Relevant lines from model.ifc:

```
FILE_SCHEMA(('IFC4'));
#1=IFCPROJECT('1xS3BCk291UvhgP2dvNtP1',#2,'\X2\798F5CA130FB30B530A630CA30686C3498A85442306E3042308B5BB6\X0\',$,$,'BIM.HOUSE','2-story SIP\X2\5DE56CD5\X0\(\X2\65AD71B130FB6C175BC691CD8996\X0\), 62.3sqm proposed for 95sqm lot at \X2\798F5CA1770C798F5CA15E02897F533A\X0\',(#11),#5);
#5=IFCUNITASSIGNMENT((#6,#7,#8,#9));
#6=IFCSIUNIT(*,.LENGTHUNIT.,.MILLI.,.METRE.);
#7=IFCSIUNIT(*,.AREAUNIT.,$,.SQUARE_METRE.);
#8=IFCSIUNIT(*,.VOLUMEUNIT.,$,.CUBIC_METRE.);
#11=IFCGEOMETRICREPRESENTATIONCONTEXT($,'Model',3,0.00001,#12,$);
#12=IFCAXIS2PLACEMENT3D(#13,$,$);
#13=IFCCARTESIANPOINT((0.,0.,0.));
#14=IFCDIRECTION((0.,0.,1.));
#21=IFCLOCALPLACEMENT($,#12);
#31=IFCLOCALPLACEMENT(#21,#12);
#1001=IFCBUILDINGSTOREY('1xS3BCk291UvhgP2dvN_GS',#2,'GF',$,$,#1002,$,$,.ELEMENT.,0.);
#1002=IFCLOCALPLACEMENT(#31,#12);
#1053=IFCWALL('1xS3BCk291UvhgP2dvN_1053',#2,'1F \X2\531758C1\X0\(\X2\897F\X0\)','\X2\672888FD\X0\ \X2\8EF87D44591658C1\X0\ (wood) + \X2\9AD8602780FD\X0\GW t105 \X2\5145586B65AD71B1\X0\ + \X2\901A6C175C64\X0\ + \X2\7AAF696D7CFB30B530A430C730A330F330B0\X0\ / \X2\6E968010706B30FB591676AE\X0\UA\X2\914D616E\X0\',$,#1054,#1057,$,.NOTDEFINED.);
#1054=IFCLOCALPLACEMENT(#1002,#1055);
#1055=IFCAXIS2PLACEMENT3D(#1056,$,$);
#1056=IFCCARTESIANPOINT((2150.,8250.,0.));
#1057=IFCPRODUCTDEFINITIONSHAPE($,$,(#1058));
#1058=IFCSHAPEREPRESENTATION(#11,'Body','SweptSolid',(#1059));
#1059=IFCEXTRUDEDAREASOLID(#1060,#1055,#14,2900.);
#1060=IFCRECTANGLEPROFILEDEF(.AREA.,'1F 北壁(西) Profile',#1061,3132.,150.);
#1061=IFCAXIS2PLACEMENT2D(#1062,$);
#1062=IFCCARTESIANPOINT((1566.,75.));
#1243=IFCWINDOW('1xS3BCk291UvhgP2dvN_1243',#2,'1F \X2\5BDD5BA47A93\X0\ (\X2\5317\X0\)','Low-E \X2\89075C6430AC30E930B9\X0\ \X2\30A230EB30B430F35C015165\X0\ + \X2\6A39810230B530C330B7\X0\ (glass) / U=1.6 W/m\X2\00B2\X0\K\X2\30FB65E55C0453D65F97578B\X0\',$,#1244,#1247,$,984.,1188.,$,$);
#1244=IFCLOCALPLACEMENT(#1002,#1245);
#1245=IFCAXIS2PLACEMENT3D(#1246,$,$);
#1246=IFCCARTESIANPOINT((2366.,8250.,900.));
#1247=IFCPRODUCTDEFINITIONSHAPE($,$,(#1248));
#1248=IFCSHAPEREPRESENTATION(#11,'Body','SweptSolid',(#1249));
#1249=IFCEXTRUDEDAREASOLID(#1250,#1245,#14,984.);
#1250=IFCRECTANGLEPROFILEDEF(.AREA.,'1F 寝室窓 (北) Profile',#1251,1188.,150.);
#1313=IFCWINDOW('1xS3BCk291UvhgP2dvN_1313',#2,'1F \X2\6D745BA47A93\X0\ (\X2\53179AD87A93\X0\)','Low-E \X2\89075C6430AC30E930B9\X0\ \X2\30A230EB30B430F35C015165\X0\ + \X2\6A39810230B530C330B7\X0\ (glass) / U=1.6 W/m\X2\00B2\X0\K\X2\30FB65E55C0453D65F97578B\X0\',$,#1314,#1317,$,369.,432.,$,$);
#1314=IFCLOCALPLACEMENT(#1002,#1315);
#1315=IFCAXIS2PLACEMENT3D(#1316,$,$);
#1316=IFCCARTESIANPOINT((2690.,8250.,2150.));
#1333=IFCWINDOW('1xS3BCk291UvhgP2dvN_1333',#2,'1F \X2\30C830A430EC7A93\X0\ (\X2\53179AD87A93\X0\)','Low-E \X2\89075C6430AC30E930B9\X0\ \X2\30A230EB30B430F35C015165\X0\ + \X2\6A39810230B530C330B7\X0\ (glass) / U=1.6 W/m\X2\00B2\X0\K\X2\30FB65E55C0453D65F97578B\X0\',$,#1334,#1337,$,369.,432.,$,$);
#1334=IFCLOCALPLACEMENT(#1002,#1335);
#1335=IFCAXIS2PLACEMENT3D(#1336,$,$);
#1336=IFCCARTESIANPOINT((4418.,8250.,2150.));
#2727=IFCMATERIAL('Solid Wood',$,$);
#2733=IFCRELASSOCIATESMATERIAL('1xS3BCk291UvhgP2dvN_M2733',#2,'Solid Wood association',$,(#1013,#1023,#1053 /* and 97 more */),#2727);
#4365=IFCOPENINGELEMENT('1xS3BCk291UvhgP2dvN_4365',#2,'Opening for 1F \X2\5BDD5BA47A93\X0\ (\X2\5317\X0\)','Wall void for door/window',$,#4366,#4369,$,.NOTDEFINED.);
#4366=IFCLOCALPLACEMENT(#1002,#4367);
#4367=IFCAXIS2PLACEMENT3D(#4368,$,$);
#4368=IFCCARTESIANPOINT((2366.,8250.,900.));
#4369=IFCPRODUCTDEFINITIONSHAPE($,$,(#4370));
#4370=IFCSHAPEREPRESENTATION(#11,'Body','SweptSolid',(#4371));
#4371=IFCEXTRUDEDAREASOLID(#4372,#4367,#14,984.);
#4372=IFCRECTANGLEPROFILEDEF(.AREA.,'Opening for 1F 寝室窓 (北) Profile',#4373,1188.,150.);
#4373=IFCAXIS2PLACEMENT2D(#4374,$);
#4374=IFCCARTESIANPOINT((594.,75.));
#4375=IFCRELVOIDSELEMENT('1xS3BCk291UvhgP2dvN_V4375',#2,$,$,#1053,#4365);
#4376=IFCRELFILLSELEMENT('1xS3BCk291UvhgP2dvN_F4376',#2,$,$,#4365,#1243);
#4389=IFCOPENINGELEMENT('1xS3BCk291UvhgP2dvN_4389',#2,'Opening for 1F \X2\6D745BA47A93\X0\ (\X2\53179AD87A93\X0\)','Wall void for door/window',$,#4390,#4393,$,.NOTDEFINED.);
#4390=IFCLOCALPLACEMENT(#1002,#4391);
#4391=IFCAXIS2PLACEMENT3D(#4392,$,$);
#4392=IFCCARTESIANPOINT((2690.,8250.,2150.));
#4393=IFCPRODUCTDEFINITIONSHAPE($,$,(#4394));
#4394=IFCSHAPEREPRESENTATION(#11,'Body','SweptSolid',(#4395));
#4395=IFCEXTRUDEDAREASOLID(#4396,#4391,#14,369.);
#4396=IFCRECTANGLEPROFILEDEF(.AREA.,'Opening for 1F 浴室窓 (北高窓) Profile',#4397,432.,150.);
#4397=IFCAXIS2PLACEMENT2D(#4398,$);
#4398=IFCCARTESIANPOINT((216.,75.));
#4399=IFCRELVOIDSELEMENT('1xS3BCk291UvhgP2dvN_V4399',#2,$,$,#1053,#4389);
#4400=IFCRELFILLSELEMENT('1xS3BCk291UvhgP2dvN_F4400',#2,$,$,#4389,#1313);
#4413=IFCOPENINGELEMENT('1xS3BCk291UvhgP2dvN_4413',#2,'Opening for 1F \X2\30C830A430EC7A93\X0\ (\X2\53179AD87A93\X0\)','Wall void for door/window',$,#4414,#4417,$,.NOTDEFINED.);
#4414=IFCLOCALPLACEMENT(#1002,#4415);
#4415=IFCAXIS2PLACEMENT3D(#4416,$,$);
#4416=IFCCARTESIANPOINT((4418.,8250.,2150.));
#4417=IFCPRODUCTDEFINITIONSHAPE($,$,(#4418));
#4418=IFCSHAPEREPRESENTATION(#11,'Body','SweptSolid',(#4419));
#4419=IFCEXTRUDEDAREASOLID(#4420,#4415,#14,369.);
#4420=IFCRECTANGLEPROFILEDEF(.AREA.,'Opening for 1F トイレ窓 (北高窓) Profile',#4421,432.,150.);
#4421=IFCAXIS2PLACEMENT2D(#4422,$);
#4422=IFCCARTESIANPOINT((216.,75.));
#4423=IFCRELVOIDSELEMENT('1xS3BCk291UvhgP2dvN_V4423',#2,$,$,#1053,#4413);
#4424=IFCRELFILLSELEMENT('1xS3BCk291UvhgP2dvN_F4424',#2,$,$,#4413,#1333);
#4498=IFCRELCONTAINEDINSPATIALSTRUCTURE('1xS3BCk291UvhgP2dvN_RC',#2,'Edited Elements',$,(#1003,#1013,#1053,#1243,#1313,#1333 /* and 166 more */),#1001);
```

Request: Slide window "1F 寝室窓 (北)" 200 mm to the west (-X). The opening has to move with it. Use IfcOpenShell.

```python
import ifcopenshell
import ifcopenshell.api.geometry
import ifcopenshell.util.placement

model = ifcopenshell.open("model.ifc")

window = model.by_guid("1xS3BCk291UvhgP2dvN_1243")
opening = window.FillsVoids[0].RelatingOpeningElement
wall = opening.VoidsElements[0].RelatingBuildingElement

wall_matrix = ifcopenshell.util.placement.get_local_placement(wall.ObjectPlacement)
shift = wall_matrix[:3, 0] * -200.0
before = ifcopenshell.util.placement.get_local_placement(window.ObjectPlacement)[:3, 3].copy()

# The window is not placed relative to its opening, so move both.
for product in (opening, window):
    matrix = ifcopenshell.util.placement.get_local_placement(product.ObjectPlacement)
    matrix[:3, 3] += shift
    ifcopenshell.api.geometry.edit_object_placement(model, product=product, matrix=matrix, is_si=False)

after = ifcopenshell.util.placement.get_local_placement(window.ObjectPlacement)[:3, 3]
print("window moved by", (after - before).round(3) + 0.0)

model.write("model_v2.ifc")
```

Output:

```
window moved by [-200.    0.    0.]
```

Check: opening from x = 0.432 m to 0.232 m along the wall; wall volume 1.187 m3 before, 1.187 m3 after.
